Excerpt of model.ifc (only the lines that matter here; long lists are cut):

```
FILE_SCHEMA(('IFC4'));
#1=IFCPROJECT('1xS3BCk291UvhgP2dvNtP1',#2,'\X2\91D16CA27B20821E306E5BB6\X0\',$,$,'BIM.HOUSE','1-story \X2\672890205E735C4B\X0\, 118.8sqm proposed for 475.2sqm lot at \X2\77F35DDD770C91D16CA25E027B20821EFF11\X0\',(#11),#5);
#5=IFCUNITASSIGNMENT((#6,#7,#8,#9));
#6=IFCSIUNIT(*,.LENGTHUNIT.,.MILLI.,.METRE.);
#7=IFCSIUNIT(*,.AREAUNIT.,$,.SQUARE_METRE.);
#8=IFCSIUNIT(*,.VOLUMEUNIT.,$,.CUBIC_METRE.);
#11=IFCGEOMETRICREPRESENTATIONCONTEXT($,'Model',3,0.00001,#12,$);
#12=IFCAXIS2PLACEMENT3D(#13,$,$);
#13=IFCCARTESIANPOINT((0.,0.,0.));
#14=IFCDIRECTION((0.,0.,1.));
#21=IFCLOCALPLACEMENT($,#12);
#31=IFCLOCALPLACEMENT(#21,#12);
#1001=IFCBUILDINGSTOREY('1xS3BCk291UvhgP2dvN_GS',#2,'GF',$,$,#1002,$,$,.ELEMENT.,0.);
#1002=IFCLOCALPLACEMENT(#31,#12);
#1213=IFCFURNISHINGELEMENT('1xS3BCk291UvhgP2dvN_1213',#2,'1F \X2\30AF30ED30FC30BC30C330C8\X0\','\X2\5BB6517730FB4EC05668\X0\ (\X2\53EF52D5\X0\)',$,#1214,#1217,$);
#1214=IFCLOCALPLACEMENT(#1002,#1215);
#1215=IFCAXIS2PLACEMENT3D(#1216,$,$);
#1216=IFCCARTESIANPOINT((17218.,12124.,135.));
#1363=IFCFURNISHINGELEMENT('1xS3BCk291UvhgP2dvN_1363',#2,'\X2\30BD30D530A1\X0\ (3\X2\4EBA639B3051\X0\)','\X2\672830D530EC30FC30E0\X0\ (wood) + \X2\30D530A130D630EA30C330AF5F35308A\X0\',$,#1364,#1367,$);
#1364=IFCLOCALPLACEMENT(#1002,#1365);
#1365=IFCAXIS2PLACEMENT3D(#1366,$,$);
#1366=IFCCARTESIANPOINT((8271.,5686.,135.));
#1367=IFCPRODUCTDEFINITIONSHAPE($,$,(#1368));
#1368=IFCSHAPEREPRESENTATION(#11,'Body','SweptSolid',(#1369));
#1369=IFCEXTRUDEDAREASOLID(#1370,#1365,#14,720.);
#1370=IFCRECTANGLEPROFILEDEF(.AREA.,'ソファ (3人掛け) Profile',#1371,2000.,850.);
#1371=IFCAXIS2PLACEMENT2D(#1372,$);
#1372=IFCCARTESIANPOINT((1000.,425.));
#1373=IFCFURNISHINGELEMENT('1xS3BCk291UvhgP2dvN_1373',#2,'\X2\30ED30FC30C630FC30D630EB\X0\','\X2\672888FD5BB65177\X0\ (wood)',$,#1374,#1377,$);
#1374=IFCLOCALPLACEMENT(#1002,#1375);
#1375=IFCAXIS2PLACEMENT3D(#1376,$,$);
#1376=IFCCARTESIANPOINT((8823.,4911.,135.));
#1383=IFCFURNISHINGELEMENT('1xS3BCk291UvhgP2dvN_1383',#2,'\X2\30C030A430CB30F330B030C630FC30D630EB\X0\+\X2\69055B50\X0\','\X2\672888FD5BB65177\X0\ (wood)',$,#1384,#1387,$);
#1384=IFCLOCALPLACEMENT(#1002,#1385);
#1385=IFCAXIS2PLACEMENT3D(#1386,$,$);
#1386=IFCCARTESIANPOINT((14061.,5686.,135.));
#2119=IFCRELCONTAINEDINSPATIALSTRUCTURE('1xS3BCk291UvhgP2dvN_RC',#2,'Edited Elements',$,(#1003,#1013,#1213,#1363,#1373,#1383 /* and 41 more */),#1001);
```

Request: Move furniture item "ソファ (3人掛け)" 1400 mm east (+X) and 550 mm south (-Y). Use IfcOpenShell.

```python
import ifcopenshell
import ifcopenshell.api.geometry
import ifcopenshell.util.placement
import ifcopenshell.util.unit

model = ifcopenshell.open("model.ifc")
unit_scale = ifcopenshell.util.unit.calculate_unit_scale(model)

item = model.by_guid("1xS3BCk291UvhgP2dvN_1363")
matrix = ifcopenshell.util.placement.get_local_placement(item.ObjectPlacement)
matrix[0, 3] += 1.4 / unit_scale
matrix[1, 3] -= 0.55 / unit_scale
ifcopenshell.api.geometry.edit_object_placement(model, product=item, matrix=matrix, is_si=False)

print(ifcopenshell.util.placement.get_local_placement(item.ObjectPlacement).round(3) + 0.0)

model.write("model-out.ifc")
```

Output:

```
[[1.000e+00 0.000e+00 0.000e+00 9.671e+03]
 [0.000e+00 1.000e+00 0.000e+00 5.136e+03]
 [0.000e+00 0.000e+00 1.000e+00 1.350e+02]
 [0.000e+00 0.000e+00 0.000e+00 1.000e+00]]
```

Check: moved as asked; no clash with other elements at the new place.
